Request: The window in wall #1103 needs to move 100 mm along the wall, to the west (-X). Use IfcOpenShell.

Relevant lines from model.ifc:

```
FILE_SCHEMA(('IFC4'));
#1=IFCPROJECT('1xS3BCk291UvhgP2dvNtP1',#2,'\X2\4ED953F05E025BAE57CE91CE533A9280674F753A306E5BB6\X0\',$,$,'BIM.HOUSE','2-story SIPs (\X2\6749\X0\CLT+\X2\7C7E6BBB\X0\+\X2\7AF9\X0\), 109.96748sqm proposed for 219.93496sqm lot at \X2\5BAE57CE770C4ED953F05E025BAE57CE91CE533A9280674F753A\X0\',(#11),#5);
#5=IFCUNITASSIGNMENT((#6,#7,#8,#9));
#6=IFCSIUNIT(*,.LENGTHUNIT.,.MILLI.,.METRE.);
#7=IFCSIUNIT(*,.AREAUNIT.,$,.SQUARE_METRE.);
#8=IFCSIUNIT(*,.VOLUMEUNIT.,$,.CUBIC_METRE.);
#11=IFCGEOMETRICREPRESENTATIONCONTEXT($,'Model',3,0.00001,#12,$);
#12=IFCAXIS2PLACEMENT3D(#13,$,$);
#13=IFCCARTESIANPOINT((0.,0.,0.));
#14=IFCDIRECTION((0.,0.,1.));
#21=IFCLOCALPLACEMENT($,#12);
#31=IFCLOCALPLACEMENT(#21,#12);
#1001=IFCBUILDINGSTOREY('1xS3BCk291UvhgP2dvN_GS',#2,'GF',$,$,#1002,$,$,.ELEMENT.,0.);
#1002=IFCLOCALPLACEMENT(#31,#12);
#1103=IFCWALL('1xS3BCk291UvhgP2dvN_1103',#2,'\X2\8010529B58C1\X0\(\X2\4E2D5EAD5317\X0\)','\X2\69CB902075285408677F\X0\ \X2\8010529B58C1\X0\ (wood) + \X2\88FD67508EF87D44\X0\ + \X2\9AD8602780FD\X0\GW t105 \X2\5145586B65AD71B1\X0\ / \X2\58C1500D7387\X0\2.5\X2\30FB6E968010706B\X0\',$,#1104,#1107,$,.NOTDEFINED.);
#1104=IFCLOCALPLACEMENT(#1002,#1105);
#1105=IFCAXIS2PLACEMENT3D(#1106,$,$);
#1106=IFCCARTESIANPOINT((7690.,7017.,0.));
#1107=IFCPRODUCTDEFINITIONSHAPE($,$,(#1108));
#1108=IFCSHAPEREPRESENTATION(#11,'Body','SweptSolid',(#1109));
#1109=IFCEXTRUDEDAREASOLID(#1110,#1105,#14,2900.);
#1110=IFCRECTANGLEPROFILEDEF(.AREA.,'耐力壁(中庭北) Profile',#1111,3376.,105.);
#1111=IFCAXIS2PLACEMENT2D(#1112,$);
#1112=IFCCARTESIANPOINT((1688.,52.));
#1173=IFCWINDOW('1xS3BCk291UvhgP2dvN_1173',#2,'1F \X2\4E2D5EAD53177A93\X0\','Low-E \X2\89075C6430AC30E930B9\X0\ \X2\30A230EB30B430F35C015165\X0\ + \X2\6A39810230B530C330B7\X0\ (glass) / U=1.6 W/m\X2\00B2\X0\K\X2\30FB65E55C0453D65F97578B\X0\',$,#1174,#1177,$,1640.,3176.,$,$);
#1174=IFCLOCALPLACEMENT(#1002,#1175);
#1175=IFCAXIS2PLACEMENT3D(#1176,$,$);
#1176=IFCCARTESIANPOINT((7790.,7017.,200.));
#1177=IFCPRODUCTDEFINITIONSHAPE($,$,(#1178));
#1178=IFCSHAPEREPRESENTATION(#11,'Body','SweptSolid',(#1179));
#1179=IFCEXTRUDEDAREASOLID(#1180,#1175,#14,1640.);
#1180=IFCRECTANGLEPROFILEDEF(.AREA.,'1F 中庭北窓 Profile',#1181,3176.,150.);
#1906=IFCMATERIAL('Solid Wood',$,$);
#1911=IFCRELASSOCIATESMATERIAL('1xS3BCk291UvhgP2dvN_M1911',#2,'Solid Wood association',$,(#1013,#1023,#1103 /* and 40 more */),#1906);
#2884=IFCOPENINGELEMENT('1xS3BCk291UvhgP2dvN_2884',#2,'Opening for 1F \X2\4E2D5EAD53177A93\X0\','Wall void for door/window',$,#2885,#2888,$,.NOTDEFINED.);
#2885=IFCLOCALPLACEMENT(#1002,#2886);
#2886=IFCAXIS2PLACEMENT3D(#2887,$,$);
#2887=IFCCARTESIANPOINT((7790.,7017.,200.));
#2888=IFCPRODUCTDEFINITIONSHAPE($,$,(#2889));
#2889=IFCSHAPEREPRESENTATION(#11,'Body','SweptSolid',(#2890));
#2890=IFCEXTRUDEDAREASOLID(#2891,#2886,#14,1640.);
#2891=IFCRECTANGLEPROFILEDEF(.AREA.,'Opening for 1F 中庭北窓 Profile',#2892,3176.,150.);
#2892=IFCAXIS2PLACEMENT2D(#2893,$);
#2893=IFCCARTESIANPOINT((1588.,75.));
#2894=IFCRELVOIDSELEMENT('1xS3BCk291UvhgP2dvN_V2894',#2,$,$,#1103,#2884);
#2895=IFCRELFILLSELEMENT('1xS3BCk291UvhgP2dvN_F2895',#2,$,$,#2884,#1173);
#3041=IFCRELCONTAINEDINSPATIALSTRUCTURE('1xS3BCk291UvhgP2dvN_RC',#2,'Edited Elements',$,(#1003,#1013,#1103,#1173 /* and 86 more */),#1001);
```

```python
import ifcopenshell
import ifcopenshell.api.geometry
import ifcopenshell.util.placement
import ifcopenshell.util.unit

model = ifcopenshell.open("model.ifc")
unit_scale = ifcopenshell.util.unit.calculate_unit_scale(model)

window = model.by_guid("1xS3BCk291UvhgP2dvN_1173")
opening = window.FillsVoids[0].RelatingOpeningElement
wall = opening.VoidsElements[0].RelatingBuildingElement

wall_matrix = ifcopenshell.util.placement.get_local_placement(wall.ObjectPlacement)
shift = wall_matrix[:3, 0] * -0.1 / unit_scale
before = ifcopenshell.util.placement.get_local_placement(window.ObjectPlacement)[:3, 3].copy()

# The window is not placed relative to its opening, so move both.
for product in (opening, window):
    matrix = ifcopenshell.util.placement.get_local_placement(product.ObjectPlacement)
    matrix[:3, 3] += shift
    ifcopenshell.api.geometry.edit_object_placement(model, product=product, matrix=matrix, is_si=False)

after = ifcopenshell.util.placement.get_local_placement(window.ObjectPlacement)[:3, 3]
print("window moved by", (after - before).round(3) + 0.0)

model.write("model_updated.ifc")
```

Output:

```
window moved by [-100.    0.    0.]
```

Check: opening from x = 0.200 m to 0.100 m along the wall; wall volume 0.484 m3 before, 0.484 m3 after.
